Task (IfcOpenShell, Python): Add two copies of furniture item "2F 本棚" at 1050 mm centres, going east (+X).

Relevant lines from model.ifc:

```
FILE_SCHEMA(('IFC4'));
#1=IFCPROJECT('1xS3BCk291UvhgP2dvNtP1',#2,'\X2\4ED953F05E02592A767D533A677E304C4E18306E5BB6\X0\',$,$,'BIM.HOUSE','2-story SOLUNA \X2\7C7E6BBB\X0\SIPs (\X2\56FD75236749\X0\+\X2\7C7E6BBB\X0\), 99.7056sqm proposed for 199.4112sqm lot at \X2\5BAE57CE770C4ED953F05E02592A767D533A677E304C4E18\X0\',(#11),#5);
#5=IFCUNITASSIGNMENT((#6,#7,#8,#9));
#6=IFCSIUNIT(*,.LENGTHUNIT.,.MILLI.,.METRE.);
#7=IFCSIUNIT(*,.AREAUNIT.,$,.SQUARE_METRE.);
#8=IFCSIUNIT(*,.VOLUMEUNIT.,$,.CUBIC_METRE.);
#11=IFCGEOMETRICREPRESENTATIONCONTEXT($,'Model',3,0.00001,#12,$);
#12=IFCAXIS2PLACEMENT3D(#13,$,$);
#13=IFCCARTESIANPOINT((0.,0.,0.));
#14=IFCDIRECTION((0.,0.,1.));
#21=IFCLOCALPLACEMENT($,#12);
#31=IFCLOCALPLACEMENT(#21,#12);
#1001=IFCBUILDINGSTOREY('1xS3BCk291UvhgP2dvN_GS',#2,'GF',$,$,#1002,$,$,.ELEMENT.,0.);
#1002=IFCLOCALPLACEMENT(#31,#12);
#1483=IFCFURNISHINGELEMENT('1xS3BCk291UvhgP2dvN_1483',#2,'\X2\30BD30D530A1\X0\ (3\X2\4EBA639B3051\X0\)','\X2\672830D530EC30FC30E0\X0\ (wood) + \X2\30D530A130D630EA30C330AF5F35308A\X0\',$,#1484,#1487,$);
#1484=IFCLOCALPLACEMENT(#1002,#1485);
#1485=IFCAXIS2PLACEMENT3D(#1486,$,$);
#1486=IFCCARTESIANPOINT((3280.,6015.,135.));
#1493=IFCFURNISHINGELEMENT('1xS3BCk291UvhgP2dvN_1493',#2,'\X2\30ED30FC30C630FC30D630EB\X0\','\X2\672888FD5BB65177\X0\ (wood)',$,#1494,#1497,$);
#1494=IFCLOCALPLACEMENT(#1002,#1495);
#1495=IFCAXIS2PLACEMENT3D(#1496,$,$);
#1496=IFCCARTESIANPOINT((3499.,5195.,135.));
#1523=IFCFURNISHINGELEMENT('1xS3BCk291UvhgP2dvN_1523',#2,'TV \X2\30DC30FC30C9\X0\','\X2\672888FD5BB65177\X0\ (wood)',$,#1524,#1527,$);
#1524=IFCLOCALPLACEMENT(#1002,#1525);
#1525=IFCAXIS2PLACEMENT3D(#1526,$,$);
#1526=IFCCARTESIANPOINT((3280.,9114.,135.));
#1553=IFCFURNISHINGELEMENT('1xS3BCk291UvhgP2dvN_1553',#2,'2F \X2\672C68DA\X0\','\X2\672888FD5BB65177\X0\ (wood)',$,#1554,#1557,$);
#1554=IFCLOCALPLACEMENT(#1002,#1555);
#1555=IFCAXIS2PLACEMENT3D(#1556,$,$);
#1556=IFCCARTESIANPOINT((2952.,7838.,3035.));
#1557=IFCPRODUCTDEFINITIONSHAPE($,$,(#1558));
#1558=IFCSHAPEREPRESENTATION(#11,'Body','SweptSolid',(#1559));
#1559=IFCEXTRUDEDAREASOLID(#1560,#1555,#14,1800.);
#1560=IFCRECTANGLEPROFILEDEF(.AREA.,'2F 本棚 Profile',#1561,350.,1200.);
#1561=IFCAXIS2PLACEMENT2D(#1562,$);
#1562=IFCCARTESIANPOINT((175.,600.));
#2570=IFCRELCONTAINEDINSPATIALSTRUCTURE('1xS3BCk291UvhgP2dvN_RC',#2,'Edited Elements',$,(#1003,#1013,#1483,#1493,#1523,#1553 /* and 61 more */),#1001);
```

```python
import numpy as np
import ifcopenshell
import ifcopenshell.api.geometry
import ifcopenshell.api.root
import ifcopenshell.util.element
import ifcopenshell.util.placement

model = ifcopenshell.open("model.ifc")


def reuse_history(source, copy):
    """copy_class also copies each property set's owner history, people and application; keep the originals."""
    for rel in copy.IsDefinedBy:
        if rel.is_a("IfcRelDefinesByProperties") and (history := rel.RelatingPropertyDefinition.OwnerHistory):
            rel.RelatingPropertyDefinition.OwnerHistory = source.OwnerHistory
            ifcopenshell.util.element.remove_deep2(model, history)


source = model.by_guid("1xS3BCk291UvhgP2dvN_1553")
base = ifcopenshell.util.placement.get_local_placement(source.ObjectPlacement)
step = np.array([1.0, 0.0, 0.0]) * 1050.0

for i in range(1, 3):
    copy = ifcopenshell.api.root.copy_class(model, product=source)
    copy.Representation = ifcopenshell.util.element.copy_deep(
        model, source.Representation, exclude=["IfcGeometricRepresentationContext", "IfcRepresentationMap"]
    )
    reuse_history(source, copy)
    matrix = base.copy()
    matrix[:3, 3] += i * step
    print("added at", matrix[:3, 3].round(3) + 0.0)
    ifcopenshell.api.geometry.edit_object_placement(model, product=copy, matrix=matrix, is_si=False)

model.write("model_edited.ifc")
```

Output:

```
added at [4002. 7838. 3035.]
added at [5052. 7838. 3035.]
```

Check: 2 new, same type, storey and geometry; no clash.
